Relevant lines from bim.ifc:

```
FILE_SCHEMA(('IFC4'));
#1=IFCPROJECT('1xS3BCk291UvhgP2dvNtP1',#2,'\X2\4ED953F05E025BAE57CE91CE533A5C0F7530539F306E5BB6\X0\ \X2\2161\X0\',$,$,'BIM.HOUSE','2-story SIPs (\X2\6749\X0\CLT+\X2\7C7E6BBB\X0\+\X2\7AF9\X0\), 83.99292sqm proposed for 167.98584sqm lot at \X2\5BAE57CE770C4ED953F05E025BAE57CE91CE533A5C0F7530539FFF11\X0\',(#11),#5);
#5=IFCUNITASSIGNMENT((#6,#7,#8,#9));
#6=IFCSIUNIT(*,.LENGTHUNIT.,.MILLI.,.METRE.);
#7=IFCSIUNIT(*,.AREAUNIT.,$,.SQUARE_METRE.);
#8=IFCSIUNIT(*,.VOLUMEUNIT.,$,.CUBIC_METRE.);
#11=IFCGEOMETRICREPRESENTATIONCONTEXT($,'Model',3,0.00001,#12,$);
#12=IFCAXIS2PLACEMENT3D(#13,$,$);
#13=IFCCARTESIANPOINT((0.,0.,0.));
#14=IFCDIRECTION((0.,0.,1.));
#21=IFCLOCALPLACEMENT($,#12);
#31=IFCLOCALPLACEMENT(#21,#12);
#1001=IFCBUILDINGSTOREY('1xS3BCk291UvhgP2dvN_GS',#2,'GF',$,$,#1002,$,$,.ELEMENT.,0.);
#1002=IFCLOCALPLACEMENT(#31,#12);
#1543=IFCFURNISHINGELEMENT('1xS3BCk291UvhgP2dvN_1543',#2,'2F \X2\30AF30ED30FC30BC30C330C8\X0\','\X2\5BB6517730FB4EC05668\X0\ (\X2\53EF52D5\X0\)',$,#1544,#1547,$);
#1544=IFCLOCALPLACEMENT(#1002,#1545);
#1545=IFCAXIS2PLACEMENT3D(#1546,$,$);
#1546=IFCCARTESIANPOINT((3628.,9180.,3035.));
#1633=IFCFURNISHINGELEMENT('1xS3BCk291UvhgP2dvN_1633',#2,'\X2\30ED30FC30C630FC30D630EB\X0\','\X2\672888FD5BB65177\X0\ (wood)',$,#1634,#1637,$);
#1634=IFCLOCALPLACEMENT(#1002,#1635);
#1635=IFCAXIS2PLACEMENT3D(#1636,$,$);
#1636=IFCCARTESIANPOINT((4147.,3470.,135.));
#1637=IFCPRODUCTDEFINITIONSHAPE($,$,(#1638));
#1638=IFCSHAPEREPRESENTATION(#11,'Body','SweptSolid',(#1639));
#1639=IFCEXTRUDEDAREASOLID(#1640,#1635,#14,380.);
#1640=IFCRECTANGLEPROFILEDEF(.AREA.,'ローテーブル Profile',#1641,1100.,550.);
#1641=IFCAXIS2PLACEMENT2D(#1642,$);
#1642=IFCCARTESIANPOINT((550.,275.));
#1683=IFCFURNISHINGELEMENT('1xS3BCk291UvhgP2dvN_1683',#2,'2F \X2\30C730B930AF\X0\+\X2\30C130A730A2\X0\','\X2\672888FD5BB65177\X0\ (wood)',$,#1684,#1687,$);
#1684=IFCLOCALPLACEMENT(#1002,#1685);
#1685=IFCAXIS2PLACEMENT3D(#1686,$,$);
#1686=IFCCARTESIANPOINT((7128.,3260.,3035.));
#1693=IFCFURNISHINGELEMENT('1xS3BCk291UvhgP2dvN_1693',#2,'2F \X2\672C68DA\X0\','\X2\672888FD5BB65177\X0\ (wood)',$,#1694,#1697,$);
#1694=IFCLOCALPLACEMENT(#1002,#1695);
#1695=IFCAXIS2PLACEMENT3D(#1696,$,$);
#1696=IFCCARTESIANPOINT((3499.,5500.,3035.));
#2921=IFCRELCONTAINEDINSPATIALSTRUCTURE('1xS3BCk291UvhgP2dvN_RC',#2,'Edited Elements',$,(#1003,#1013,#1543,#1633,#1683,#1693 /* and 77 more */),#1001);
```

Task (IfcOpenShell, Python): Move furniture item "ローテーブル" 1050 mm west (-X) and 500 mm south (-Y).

```python
import ifcopenshell
import ifcopenshell.api.geometry
import ifcopenshell.util.placement
import ifcopenshell.util.unit

model = ifcopenshell.open("bim.ifc")
unit_scale = ifcopenshell.util.unit.calculate_unit_scale(model)

item = model.by_id(1633)
matrix = ifcopenshell.util.placement.get_local_placement(item.ObjectPlacement)
matrix[0, 3] -= 1.05 / unit_scale
matrix[1, 3] -= 0.5 / unit_scale
ifcopenshell.api.geometry.edit_object_placement(model, product=item, matrix=matrix, is_si=False)

print(ifcopenshell.util.placement.get_local_placement(item.ObjectPlacement).round(3) + 0.0)

model.write("bim_updated.ifc")
```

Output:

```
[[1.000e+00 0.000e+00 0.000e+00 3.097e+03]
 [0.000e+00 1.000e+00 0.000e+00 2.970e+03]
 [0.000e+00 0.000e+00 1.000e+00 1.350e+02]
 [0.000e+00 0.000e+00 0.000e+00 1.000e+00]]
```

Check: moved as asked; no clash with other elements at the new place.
